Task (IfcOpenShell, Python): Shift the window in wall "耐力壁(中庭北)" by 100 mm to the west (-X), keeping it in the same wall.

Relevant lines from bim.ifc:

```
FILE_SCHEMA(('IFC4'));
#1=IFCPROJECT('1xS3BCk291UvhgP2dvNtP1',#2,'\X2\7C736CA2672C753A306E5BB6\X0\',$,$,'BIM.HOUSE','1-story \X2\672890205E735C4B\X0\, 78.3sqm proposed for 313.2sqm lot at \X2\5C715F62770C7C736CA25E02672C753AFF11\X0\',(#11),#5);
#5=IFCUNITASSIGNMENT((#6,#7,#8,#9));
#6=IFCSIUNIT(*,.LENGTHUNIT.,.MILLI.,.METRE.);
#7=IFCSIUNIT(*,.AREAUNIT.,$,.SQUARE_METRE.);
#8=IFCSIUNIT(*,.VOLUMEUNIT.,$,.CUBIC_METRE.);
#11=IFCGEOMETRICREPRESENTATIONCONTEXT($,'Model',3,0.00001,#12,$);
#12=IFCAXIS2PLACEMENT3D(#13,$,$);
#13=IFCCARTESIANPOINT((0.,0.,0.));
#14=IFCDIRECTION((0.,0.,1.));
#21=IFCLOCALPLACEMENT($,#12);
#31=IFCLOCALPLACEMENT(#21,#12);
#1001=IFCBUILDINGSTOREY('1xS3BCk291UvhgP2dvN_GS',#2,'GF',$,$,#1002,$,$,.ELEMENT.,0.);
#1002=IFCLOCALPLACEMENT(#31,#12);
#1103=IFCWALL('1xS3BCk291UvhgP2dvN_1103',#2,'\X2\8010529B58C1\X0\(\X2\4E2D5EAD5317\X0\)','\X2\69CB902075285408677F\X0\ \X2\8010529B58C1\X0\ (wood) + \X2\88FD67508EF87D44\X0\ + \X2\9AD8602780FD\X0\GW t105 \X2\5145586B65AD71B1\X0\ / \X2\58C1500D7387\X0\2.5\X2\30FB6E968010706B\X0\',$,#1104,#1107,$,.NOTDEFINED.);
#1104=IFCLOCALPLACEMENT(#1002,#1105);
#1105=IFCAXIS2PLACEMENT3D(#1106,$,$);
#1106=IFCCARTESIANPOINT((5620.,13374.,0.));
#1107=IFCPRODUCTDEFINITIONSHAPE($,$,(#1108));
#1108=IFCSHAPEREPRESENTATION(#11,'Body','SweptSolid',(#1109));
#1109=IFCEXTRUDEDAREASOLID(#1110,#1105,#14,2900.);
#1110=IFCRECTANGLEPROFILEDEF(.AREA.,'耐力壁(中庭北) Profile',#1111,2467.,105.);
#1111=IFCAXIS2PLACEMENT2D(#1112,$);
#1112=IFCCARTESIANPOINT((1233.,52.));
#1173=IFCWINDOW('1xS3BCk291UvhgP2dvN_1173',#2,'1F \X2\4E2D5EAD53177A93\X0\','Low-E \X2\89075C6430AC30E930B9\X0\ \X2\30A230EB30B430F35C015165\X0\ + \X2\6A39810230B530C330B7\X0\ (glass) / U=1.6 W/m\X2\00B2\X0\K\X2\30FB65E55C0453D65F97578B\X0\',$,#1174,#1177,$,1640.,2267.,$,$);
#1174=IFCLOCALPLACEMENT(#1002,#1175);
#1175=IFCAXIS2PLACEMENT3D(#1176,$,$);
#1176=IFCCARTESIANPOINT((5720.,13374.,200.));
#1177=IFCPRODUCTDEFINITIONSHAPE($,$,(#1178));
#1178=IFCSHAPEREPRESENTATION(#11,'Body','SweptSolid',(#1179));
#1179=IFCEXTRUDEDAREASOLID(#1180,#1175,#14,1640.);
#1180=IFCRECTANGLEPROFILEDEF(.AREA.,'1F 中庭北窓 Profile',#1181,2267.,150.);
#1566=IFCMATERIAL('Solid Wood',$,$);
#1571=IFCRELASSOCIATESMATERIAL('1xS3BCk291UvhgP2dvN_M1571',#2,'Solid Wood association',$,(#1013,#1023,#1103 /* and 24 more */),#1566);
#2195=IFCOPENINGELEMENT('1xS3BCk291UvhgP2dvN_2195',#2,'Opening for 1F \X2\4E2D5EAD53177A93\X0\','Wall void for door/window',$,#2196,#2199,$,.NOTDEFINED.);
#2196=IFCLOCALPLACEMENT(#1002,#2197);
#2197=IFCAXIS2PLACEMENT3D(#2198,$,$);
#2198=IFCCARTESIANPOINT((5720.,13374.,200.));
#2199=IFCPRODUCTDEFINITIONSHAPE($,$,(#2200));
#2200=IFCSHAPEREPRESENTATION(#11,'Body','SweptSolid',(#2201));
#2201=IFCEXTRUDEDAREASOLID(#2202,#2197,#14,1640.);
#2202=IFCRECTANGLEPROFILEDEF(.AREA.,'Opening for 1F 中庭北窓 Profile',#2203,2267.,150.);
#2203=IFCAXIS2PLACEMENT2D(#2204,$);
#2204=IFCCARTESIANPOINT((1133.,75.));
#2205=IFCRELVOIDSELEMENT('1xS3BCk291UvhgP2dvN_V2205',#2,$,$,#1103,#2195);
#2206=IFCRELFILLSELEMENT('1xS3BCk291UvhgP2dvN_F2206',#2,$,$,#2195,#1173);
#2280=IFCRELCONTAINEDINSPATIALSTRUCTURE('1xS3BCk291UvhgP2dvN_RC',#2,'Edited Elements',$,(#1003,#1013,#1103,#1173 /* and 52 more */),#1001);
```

```python
import ifcopenshell
import ifcopenshell.api.geometry
import ifcopenshell.util.placement
import ifcopenshell.util.unit

model = ifcopenshell.open("bim.ifc")
unit_scale = ifcopenshell.util.unit.calculate_unit_scale(model)

window = model.by_guid("1xS3BCk291UvhgP2dvN_1173")
opening = window.FillsVoids[0].RelatingOpeningElement
wall = opening.VoidsElements[0].RelatingBuildingElement

wall_matrix = ifcopenshell.util.placement.get_local_placement(wall.ObjectPlacement)
shift = wall_matrix[:3, 0] * -0.1 / unit_scale
before = ifcopenshell.util.placement.get_local_placement(window.ObjectPlacement)[:3, 3].copy()

# The window is not placed relative to its opening, so move both.
for product in (opening, window):
    matrix = ifcopenshell.util.placement.get_local_placement(product.ObjectPlacement)
    matrix[:3, 3] += shift
    ifcopenshell.api.geometry.edit_object_placement(model, product=product, matrix=matrix, is_si=False)

after = ifcopenshell.util.placement.get_local_placement(window.ObjectPlacement)[:3, 3]
print("window moved by", (after - before).round(3) + 0.0)

model.write("bim-out.ifc")
```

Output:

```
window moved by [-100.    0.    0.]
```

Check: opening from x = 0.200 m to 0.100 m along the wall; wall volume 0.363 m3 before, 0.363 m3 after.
